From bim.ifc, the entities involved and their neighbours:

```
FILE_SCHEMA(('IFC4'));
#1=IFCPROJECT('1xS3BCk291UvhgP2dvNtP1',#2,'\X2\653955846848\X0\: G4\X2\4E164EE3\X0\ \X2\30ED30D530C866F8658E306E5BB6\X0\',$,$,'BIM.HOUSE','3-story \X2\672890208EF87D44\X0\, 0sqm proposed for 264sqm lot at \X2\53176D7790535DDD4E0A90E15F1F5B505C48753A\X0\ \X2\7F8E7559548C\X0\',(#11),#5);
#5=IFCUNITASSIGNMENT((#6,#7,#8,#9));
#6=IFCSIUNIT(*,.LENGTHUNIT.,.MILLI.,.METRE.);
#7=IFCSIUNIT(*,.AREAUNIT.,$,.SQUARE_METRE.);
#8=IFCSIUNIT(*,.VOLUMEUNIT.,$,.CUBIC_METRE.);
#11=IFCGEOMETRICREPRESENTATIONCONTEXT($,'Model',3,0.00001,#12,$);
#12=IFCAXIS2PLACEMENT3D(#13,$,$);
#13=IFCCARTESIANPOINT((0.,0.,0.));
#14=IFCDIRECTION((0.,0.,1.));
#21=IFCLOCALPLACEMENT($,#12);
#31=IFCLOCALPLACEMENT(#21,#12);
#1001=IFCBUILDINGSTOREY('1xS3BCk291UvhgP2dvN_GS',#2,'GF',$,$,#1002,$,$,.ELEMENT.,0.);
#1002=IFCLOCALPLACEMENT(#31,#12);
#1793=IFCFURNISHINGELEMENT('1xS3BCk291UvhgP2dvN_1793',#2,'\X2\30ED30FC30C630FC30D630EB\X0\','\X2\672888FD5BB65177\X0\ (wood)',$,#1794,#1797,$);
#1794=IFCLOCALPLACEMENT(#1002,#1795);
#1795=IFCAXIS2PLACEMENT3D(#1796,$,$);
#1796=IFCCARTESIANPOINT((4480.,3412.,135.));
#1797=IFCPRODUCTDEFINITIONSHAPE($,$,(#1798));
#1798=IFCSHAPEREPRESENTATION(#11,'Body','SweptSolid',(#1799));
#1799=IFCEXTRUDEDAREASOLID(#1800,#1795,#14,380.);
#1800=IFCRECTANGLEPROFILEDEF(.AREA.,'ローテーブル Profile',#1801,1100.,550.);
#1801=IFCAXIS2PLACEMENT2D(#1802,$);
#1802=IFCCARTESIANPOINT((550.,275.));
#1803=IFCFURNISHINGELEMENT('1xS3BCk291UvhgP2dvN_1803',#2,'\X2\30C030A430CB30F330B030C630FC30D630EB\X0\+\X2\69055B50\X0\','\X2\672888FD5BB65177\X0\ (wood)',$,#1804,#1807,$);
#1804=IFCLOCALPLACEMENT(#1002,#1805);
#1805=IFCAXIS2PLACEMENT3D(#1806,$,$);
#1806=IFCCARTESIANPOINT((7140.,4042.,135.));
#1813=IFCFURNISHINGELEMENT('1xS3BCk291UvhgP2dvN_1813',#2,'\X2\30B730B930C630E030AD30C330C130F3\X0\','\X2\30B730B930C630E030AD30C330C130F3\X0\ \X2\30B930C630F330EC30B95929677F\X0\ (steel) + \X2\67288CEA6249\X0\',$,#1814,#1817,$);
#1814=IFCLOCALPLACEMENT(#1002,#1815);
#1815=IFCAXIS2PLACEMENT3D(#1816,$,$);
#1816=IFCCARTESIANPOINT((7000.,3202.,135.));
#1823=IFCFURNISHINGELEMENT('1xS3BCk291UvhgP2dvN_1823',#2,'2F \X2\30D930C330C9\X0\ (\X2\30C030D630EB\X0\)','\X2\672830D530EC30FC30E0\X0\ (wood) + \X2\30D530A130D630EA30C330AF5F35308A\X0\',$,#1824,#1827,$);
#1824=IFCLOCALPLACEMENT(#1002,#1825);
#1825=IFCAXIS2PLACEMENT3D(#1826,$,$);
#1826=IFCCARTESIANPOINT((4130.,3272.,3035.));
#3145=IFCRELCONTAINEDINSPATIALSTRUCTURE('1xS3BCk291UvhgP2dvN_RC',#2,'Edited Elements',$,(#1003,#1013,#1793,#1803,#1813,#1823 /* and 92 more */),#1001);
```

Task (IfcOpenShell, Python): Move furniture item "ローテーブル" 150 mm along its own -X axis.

```python
import ifcopenshell
import ifcopenshell.api.geometry
import ifcopenshell.util.placement
import ifcopenshell.util.unit

model = ifcopenshell.open("bim.ifc")
unit_scale = ifcopenshell.util.unit.calculate_unit_scale(model)

item = model.by_guid("1xS3BCk291UvhgP2dvN_1793")
matrix = ifcopenshell.util.placement.get_local_placement(item.ObjectPlacement)
matrix[:3, 3] -= matrix[:3, 0] * 0.15 / unit_scale
ifcopenshell.api.geometry.edit_object_placement(model, product=item, matrix=matrix, is_si=False)

print(ifcopenshell.util.placement.get_local_placement(item.ObjectPlacement).round(3) + 0.0)

model.write("bim_rev.ifc")
```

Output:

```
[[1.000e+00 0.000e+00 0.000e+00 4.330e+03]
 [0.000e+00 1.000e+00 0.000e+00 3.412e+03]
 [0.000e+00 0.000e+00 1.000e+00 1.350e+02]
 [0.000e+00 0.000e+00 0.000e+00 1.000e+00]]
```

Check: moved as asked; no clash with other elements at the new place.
